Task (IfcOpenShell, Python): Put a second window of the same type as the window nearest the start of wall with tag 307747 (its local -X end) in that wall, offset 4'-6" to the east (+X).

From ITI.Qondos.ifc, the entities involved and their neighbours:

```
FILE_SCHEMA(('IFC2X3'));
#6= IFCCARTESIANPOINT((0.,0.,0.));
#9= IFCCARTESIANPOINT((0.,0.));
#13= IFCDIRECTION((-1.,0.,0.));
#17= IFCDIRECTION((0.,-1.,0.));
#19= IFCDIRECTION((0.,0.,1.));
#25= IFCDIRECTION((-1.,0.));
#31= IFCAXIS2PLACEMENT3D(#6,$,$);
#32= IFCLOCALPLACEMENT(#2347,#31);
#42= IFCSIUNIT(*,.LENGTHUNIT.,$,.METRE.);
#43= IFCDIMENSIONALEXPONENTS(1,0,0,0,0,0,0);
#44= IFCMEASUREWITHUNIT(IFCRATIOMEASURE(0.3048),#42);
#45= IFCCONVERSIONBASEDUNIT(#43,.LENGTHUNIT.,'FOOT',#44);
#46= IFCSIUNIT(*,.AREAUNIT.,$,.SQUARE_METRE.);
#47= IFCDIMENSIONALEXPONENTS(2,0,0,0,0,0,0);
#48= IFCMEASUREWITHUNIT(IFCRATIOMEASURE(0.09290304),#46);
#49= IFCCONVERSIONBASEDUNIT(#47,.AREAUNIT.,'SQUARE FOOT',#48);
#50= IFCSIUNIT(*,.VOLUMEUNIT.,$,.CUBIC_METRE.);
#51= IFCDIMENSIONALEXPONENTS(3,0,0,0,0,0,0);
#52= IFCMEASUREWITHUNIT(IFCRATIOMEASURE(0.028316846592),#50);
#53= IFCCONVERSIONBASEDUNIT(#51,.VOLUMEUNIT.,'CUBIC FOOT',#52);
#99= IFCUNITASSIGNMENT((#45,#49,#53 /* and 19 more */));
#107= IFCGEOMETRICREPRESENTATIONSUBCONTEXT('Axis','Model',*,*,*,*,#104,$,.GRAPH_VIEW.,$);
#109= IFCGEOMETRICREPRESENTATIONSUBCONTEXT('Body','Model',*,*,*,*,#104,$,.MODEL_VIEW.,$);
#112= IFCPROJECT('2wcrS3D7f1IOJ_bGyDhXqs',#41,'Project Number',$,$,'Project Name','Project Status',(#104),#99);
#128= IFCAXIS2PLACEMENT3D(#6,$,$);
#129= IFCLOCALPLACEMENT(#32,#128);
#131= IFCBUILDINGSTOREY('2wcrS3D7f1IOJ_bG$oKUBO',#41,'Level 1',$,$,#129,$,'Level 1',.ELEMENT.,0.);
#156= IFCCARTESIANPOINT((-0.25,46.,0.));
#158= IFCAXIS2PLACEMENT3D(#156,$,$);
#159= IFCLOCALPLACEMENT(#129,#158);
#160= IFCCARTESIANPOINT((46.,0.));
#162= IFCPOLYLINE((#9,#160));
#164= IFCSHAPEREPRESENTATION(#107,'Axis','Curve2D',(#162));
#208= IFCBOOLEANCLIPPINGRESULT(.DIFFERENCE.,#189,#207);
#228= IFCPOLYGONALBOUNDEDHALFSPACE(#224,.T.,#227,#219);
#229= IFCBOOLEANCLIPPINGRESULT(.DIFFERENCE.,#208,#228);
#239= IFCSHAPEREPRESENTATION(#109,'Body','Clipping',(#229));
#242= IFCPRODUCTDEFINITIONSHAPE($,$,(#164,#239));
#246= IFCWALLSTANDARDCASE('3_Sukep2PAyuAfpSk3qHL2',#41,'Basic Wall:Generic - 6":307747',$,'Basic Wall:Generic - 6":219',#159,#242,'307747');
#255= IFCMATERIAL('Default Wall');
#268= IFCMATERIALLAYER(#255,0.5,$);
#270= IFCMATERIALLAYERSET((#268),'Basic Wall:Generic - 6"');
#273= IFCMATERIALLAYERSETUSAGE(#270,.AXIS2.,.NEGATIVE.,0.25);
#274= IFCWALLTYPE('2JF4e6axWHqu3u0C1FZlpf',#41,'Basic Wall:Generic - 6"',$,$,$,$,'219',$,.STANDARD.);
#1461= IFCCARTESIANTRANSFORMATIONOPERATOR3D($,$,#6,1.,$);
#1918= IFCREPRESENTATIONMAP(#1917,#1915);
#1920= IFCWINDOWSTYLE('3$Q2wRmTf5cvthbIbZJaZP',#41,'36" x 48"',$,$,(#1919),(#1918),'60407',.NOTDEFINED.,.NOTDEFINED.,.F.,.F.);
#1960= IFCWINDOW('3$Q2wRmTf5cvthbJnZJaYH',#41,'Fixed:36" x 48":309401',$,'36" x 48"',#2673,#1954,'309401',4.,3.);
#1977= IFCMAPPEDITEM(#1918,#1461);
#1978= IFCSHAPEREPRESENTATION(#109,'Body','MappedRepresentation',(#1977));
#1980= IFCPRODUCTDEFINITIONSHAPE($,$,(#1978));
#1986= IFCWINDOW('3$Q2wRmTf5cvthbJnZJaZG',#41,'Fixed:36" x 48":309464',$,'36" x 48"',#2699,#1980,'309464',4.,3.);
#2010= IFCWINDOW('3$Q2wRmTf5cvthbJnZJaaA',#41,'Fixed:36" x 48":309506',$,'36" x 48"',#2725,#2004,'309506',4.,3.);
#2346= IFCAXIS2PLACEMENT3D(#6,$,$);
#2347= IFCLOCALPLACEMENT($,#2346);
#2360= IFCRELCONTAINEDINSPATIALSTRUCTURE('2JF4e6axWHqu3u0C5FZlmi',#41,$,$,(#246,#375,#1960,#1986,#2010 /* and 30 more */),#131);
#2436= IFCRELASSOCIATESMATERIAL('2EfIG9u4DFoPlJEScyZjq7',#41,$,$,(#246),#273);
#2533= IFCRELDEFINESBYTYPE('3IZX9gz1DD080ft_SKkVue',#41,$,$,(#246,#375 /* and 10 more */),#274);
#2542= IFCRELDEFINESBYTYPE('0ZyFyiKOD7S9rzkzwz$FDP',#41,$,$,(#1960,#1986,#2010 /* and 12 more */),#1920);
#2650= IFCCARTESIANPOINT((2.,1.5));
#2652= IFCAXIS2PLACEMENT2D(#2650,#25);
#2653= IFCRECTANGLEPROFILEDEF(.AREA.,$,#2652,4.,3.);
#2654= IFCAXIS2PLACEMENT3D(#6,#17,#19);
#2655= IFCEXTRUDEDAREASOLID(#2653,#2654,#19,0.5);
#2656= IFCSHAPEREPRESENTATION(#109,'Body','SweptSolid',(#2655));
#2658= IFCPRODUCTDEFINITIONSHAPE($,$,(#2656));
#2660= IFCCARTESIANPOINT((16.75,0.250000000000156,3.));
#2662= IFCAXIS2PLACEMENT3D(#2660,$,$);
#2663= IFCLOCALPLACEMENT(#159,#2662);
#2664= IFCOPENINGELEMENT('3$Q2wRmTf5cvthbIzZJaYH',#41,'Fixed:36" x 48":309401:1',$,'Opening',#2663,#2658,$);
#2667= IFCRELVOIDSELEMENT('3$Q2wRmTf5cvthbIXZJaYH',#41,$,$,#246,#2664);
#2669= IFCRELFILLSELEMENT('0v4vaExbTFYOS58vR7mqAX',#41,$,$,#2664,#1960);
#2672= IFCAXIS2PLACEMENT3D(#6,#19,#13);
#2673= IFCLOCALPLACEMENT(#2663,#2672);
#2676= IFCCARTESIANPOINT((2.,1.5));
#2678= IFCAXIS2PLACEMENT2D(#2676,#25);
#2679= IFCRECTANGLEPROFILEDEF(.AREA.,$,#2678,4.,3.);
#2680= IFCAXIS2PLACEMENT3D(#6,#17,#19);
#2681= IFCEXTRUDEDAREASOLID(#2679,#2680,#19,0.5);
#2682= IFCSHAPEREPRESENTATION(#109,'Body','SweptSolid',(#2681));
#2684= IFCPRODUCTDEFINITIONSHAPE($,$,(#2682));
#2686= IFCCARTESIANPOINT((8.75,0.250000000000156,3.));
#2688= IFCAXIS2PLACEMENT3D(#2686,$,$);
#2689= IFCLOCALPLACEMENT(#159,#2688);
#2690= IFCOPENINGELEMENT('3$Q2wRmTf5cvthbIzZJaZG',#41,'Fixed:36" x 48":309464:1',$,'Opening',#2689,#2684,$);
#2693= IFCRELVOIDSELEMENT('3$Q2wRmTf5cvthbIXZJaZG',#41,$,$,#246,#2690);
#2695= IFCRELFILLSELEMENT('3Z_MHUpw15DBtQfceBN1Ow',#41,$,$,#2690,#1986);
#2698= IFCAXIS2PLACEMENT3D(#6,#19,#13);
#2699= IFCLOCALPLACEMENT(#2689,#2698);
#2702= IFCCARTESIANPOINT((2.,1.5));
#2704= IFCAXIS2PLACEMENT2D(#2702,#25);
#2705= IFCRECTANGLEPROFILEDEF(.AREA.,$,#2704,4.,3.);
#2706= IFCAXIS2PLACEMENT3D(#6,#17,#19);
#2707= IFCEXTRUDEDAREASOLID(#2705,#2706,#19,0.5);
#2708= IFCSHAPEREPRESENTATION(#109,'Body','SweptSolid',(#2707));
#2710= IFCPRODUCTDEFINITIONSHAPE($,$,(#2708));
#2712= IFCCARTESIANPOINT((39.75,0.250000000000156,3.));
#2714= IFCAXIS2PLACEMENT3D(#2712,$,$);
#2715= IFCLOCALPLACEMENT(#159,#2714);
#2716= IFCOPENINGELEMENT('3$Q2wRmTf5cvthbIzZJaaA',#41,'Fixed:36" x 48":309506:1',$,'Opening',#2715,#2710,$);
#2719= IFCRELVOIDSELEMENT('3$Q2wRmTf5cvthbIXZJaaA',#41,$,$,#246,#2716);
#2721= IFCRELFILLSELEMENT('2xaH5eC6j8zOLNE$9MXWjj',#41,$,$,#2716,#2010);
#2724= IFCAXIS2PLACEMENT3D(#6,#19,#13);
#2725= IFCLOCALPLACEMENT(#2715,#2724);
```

```python
import ifcopenshell
import ifcopenshell.api.feature
import ifcopenshell.api.geometry
import ifcopenshell.api.root
import ifcopenshell.geom
import ifcopenshell.util.element
import ifcopenshell.util.placement
import ifcopenshell.util.shape
import ifcopenshell.util.unit

model = ifcopenshell.open("ITI.Qondos.ifc")
unit_scale = ifcopenshell.util.unit.calculate_unit_scale(model)
settings = ifcopenshell.geom.settings()


def volume(element):
    """Net volume in cubic metres, openings subtracted."""
    shape = ifcopenshell.geom.create_shape(settings, element)
    return ifcopenshell.util.shape.get_volume(shape.geometry)


def reuse_history(source, copy):
    """copy_class also copies each property set's owner history, people and application; keep the originals."""
    for rel in copy.IsDefinedBy:
        if rel.is_a("IfcRelDefinesByProperties") and (history := rel.RelatingPropertyDefinition.OwnerHistory):
            rel.RelatingPropertyDefinition.OwnerHistory = source.OwnerHistory
            ifcopenshell.util.element.remove_deep2(model, history)


window = model.by_guid("3$Q2wRmTf5cvthbJnZJaZG")
opening = window.FillsVoids[0].RelatingOpeningElement
wall = opening.VoidsElements[0].RelatingBuildingElement
before = volume(wall)
shift = ifcopenshell.util.placement.get_local_placement(wall.ObjectPlacement)[:3, 0] * 54 * 0.0254 / unit_scale

# copy_class copies the void relationship, type, container and properties, but no geometry.
new_opening = ifcopenshell.api.root.copy_class(model, product=opening)
new_opening.Representation = ifcopenshell.util.element.copy_deep(
    model, opening.Representation, exclude=["IfcGeometricRepresentationContext", "IfcRepresentationMap"]
)
new_opening.Name = 'Fixed:36" x 48"'
new_window = ifcopenshell.api.root.copy_class(model, product=window)
new_window.Representation = ifcopenshell.util.element.copy_deep(
    model, window.Representation, exclude=["IfcGeometricRepresentationContext", "IfcRepresentationMap"]
)
new_window.Name = 'Fixed:36" x 48"'
new_window.Tag = None
reuse_history(window, new_window)
fills = ifcopenshell.api.feature.add_filling(model, opening=new_opening, element=new_window)
fills.OwnerHistory = new_window.OwnerHistory  # required in IFC2X3

for old, new in ((opening, new_opening), (window, new_window)):
    matrix = ifcopenshell.util.placement.get_local_placement(old.ObjectPlacement)
    matrix[:3, 3] += shift
    ifcopenshell.api.geometry.edit_object_placement(model, product=new, matrix=matrix, is_si=False)

after = volume(wall)

print(f"wall volume {before:.3f} -> {after:.3f} m3")

model.write("ITI.Qondos_v2.ifc")
```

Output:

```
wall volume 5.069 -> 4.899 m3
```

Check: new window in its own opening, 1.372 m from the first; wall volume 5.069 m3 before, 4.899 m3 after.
